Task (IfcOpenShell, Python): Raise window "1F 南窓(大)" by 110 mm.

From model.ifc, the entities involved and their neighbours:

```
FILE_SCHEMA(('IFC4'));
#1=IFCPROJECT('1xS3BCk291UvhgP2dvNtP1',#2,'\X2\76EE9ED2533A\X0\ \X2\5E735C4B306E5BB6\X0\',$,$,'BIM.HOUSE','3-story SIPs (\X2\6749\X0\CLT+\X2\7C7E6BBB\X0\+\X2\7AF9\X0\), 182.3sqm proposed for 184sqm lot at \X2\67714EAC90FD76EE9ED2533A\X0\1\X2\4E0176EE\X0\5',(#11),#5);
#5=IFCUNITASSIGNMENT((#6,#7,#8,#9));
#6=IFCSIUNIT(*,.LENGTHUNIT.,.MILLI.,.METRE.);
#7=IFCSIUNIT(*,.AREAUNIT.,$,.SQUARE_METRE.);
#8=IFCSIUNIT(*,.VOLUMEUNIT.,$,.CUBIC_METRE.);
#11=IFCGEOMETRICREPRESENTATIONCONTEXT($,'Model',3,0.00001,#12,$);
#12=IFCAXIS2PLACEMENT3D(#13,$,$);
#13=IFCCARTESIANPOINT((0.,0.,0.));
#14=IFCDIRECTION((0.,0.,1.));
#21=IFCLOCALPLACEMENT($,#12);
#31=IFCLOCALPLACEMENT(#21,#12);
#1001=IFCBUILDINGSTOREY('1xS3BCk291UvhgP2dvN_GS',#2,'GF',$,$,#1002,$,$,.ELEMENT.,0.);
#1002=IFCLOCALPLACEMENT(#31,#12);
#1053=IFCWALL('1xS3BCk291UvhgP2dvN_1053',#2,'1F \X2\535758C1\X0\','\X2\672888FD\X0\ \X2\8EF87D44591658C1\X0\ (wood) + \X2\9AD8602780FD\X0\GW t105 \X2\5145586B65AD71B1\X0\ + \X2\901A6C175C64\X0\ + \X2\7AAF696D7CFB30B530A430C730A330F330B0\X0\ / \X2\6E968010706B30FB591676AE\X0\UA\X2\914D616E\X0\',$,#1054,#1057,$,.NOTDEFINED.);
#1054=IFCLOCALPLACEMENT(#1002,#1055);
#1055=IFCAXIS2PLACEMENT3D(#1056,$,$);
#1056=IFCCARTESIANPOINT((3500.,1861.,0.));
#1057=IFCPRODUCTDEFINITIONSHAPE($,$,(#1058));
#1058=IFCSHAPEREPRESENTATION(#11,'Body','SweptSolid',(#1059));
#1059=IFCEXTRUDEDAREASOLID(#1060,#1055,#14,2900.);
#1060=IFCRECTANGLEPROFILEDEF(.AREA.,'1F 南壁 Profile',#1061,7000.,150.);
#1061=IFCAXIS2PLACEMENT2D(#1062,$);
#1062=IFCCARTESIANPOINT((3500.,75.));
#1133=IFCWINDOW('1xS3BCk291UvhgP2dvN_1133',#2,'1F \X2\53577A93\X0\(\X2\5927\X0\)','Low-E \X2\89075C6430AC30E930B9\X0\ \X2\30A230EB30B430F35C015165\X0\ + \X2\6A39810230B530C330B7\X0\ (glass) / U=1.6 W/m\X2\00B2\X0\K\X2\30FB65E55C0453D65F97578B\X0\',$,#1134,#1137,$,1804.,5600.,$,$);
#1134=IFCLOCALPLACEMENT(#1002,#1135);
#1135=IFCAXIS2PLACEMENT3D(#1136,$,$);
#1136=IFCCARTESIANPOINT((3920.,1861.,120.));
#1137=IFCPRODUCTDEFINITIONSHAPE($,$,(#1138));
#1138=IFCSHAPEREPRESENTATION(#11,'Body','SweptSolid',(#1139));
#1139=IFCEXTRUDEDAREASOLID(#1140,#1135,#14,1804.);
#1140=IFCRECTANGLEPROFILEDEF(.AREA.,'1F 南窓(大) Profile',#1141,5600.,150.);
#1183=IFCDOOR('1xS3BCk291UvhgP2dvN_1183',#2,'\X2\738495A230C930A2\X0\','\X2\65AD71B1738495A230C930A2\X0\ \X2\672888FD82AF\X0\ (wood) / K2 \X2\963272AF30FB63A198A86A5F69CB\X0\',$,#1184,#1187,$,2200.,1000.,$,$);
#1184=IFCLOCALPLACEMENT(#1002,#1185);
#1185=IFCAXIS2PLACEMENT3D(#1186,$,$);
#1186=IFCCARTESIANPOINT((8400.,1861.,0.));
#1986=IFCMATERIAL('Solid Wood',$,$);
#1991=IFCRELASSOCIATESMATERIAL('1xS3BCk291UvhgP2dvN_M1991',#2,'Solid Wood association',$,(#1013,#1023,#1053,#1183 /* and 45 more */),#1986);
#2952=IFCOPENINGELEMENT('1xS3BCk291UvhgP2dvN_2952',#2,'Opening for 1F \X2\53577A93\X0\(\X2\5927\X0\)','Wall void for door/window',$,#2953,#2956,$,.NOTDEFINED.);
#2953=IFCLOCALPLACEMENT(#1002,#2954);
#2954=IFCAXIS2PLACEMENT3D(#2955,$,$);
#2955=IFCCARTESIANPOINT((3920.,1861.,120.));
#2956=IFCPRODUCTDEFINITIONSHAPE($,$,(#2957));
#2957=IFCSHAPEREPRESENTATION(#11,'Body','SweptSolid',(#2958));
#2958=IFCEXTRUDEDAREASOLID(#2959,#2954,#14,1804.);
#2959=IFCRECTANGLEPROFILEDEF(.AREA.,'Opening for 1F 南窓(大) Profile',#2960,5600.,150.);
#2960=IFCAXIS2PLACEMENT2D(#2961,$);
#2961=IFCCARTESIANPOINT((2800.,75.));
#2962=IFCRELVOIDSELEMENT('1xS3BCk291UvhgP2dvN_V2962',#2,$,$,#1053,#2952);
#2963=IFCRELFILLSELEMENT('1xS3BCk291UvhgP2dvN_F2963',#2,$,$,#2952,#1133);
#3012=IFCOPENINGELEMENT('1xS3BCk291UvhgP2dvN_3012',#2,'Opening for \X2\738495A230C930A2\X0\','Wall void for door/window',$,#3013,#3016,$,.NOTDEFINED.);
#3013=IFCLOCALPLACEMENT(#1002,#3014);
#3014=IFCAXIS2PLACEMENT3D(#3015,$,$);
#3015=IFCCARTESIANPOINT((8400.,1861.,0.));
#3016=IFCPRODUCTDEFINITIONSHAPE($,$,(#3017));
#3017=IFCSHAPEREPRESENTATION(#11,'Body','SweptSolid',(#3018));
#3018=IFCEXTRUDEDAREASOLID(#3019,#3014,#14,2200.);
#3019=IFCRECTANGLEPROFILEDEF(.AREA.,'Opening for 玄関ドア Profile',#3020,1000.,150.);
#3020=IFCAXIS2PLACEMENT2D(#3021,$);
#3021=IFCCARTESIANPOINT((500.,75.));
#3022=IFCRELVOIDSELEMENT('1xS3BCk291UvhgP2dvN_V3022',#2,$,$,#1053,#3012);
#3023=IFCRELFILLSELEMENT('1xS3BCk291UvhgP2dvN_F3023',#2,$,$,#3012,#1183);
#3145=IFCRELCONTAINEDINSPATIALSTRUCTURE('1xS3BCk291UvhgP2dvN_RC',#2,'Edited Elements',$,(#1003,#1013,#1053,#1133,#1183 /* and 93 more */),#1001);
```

```python
import numpy as np
import ifcopenshell
import ifcopenshell.api.geometry
import ifcopenshell.util.placement
import ifcopenshell.util.unit

model = ifcopenshell.open("model.ifc")
unit_scale = ifcopenshell.util.unit.calculate_unit_scale(model)

window = model.by_id(1133)
opening = window.FillsVoids[0].RelatingOpeningElement
dz = 110.0

shift = np.array([0.0, 0.0, dz])
# The window is not placed relative to its opening, so move both.
for product in (opening, window):
    matrix = ifcopenshell.util.placement.get_local_placement(product.ObjectPlacement)
    matrix[:3, 3] += shift
    ifcopenshell.api.geometry.edit_object_placement(model, product=product, matrix=matrix, is_si=False)

print(f"moved by {dz * unit_scale:+.3f} m")

model.write("model_edited.ifc")
```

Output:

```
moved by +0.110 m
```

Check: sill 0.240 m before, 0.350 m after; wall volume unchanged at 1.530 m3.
